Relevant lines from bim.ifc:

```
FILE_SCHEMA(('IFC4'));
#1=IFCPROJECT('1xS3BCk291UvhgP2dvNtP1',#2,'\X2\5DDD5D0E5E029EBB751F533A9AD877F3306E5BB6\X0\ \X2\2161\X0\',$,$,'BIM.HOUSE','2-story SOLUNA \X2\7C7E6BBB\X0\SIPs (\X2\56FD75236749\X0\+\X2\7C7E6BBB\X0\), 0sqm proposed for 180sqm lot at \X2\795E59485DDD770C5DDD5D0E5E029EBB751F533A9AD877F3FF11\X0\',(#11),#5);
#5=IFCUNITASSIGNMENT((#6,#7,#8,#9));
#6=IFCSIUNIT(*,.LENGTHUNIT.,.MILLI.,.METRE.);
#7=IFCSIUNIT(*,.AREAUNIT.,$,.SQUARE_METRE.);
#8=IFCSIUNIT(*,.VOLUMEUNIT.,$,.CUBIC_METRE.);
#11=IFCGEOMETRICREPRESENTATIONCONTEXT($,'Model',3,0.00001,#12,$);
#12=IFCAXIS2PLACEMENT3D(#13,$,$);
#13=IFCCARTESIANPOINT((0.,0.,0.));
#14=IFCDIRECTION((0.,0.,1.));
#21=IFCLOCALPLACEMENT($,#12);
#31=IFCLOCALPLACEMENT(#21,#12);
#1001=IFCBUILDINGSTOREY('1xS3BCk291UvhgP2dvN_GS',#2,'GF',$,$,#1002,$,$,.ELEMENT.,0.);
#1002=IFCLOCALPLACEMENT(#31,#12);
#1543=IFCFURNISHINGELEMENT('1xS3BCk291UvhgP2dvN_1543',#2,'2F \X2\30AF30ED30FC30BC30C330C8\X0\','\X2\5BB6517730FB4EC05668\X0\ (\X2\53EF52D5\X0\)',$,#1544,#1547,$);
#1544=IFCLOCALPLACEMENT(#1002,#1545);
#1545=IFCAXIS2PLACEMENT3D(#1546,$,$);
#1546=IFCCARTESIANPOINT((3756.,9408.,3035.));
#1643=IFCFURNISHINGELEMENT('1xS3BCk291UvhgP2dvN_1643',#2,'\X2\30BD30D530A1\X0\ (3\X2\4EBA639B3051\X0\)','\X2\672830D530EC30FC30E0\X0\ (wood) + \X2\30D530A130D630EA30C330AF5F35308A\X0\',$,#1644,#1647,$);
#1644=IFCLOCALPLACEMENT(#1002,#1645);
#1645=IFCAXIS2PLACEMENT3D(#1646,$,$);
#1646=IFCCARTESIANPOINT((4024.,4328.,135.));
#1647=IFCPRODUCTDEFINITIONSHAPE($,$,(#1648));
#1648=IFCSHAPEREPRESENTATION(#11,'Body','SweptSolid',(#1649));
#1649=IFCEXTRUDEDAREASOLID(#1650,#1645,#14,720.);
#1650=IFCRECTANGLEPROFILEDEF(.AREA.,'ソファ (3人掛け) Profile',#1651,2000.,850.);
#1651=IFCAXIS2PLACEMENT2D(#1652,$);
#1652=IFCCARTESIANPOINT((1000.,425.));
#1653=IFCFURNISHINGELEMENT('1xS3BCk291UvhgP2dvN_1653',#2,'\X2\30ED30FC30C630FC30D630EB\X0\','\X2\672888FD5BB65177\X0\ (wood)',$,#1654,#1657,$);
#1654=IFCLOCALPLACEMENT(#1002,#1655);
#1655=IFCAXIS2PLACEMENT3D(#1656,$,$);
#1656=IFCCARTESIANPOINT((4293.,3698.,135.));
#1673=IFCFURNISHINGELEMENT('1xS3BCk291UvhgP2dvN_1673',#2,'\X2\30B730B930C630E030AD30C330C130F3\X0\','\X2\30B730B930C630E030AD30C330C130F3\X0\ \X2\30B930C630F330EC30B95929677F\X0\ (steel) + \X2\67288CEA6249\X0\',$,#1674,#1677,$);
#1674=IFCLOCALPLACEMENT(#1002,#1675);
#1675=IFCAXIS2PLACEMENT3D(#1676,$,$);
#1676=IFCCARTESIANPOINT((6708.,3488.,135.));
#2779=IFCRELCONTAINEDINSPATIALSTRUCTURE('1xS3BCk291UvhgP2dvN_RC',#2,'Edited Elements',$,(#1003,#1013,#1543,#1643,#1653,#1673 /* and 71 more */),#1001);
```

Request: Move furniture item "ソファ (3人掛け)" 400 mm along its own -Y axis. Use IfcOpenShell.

```python
import ifcopenshell
import ifcopenshell.api.geometry
import ifcopenshell.util.placement
import ifcopenshell.util.unit

model = ifcopenshell.open("bim.ifc")
unit_scale = ifcopenshell.util.unit.calculate_unit_scale(model)

item = model.by_id(1643)
matrix = ifcopenshell.util.placement.get_local_placement(item.ObjectPlacement)
matrix[:3, 3] -= matrix[:3, 1] * 0.4 / unit_scale
ifcopenshell.api.geometry.edit_object_placement(model, product=item, matrix=matrix, is_si=False)

print(ifcopenshell.util.placement.get_local_placement(item.ObjectPlacement).round(3) + 0.0)

model.write("bim-out.ifc")
```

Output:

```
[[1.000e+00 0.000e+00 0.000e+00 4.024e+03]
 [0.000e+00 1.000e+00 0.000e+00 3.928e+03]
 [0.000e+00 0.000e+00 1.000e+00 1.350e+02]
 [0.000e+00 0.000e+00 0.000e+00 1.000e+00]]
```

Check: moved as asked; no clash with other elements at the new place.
